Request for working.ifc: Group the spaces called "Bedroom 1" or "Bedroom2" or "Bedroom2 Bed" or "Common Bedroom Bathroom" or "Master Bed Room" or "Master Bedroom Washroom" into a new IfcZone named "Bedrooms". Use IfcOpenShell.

First a look at what the model holds.

```python
import ifcopenshell

model = ifcopenshell.open("working.ifc")
print(model.schema)
seen = {}
for space in model.by_type("IfcSpace"):
    seen[space.Name] = seen.get(space.Name, 0) + 1
for name, count in sorted(seen.items(), key=str):
    print(count, "x", name)
print("zones:", [z.Name for z in model.by_type("IfcZone")][:20])
```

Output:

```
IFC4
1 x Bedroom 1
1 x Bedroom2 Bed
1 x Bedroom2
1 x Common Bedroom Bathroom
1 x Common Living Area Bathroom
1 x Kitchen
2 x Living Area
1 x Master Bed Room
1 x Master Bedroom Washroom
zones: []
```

```python
import ifcopenshell
import ifcopenshell.api.group
import ifcopenshell.api.root

model = ifcopenshell.open("working.ifc")

names = {"Bedroom 1", "Bedroom2", "Bedroom2 Bed", "Common Bedroom Bathroom", "Master Bed Room", "Master Bedroom Washroom"}
spaces = [s for s in model.by_type("IfcSpace") if s.Name in names]

zone = ifcopenshell.api.root.create_entity(model, ifc_class="IfcZone", name="Bedrooms")
ifcopenshell.api.group.assign_group(model, products=spaces, group=zone)
print(len(spaces), "spaces in", zone.Name)

model.write("working_v2.ifc")
```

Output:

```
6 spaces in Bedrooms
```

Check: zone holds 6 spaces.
